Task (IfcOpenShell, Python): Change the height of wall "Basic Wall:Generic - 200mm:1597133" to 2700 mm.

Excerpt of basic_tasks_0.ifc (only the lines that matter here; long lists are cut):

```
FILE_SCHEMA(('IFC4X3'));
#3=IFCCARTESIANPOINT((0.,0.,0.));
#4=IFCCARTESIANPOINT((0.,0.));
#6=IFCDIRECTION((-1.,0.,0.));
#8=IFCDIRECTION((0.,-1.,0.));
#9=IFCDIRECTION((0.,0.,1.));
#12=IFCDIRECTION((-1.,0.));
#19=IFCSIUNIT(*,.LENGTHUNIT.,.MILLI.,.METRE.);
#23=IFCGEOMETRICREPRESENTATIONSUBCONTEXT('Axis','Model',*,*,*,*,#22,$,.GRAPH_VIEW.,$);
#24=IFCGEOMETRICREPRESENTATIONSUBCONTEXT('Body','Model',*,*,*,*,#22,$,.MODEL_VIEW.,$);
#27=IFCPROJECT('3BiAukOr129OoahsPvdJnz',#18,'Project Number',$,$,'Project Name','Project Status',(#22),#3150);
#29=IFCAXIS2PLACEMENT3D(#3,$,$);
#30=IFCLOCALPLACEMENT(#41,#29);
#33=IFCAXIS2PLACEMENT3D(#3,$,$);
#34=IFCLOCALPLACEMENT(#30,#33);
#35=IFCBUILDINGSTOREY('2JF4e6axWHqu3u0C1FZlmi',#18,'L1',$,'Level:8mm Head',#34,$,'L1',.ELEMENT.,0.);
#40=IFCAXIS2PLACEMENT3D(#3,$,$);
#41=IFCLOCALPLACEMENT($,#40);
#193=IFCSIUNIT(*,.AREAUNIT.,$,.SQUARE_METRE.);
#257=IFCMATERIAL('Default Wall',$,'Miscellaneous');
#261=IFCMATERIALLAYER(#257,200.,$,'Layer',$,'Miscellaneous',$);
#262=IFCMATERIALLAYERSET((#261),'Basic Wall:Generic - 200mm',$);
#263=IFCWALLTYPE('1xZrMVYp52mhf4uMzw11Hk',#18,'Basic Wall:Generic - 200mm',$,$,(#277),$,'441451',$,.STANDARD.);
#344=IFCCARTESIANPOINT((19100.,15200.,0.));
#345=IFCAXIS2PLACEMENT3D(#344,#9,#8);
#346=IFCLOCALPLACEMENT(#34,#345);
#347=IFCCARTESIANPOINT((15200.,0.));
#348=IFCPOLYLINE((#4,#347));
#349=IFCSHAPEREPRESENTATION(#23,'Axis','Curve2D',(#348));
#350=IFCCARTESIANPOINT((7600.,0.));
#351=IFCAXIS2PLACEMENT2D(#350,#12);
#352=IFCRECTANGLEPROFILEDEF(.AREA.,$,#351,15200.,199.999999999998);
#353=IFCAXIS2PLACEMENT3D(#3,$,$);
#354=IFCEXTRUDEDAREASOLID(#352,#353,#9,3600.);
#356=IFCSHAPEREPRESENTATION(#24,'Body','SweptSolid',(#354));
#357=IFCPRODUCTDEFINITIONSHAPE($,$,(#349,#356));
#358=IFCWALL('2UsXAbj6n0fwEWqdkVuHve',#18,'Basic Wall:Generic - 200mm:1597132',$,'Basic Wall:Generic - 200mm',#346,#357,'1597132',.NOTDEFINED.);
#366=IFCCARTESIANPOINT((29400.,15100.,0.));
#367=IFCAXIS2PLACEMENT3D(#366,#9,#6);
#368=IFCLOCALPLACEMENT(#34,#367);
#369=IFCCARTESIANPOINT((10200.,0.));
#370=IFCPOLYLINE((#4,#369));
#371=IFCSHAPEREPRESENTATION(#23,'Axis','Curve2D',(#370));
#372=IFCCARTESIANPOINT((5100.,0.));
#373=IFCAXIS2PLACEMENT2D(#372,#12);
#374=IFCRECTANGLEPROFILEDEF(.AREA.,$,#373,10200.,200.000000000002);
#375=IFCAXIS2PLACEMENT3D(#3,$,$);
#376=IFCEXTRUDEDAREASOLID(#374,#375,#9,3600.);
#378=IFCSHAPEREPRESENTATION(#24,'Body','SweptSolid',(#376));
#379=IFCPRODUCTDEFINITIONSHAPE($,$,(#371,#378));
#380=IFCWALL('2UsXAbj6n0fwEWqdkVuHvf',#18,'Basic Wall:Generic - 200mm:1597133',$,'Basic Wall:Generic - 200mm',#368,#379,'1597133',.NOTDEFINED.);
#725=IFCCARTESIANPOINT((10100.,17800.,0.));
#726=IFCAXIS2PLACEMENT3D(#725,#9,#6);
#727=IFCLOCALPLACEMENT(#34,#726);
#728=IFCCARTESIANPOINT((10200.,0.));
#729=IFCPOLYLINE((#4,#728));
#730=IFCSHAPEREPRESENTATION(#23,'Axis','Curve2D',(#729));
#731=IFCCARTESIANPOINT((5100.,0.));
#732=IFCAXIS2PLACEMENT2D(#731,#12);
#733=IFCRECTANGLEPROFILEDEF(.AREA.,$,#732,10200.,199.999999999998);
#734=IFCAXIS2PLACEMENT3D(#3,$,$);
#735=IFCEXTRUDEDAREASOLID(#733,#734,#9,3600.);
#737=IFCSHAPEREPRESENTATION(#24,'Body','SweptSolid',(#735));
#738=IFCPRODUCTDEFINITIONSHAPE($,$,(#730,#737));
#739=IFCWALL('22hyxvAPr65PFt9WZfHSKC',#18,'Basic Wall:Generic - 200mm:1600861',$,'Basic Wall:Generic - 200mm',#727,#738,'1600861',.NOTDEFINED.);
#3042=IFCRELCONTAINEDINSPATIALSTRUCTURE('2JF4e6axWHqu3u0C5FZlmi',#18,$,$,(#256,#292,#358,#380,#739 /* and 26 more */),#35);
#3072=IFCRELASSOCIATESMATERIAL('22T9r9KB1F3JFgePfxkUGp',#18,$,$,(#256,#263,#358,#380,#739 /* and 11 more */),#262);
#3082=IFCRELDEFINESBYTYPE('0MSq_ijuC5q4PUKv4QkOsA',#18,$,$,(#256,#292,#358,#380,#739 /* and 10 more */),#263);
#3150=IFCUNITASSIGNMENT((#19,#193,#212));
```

```python
import ifcopenshell
import ifcopenshell.geom
import ifcopenshell.util.representation
import ifcopenshell.util.shape

model = ifcopenshell.open("basic_tasks_0.ifc")
settings = ifcopenshell.geom.settings()


def volume(element):
    """Net volume in cubic metres, openings subtracted."""
    shape = ifcopenshell.geom.create_shape(settings, element)
    return ifcopenshell.util.shape.get_volume(shape.geometry)


wall = model.by_id(380)
before = volume(wall)

body = ifcopenshell.util.representation.get_representation(wall, "Model", "Body")
solid = body.Items[0]
old_height = solid.Depth
solid.Depth = 2700.0
after = volume(wall)

print(f"height {old_height:g} -> {solid.Depth:g}, volume {before:.3f} -> {after:.3f} m3")

model.write("basic_tasks_0_updated.ifc")
```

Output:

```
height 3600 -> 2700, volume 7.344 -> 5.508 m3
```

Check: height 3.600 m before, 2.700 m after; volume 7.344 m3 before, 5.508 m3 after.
